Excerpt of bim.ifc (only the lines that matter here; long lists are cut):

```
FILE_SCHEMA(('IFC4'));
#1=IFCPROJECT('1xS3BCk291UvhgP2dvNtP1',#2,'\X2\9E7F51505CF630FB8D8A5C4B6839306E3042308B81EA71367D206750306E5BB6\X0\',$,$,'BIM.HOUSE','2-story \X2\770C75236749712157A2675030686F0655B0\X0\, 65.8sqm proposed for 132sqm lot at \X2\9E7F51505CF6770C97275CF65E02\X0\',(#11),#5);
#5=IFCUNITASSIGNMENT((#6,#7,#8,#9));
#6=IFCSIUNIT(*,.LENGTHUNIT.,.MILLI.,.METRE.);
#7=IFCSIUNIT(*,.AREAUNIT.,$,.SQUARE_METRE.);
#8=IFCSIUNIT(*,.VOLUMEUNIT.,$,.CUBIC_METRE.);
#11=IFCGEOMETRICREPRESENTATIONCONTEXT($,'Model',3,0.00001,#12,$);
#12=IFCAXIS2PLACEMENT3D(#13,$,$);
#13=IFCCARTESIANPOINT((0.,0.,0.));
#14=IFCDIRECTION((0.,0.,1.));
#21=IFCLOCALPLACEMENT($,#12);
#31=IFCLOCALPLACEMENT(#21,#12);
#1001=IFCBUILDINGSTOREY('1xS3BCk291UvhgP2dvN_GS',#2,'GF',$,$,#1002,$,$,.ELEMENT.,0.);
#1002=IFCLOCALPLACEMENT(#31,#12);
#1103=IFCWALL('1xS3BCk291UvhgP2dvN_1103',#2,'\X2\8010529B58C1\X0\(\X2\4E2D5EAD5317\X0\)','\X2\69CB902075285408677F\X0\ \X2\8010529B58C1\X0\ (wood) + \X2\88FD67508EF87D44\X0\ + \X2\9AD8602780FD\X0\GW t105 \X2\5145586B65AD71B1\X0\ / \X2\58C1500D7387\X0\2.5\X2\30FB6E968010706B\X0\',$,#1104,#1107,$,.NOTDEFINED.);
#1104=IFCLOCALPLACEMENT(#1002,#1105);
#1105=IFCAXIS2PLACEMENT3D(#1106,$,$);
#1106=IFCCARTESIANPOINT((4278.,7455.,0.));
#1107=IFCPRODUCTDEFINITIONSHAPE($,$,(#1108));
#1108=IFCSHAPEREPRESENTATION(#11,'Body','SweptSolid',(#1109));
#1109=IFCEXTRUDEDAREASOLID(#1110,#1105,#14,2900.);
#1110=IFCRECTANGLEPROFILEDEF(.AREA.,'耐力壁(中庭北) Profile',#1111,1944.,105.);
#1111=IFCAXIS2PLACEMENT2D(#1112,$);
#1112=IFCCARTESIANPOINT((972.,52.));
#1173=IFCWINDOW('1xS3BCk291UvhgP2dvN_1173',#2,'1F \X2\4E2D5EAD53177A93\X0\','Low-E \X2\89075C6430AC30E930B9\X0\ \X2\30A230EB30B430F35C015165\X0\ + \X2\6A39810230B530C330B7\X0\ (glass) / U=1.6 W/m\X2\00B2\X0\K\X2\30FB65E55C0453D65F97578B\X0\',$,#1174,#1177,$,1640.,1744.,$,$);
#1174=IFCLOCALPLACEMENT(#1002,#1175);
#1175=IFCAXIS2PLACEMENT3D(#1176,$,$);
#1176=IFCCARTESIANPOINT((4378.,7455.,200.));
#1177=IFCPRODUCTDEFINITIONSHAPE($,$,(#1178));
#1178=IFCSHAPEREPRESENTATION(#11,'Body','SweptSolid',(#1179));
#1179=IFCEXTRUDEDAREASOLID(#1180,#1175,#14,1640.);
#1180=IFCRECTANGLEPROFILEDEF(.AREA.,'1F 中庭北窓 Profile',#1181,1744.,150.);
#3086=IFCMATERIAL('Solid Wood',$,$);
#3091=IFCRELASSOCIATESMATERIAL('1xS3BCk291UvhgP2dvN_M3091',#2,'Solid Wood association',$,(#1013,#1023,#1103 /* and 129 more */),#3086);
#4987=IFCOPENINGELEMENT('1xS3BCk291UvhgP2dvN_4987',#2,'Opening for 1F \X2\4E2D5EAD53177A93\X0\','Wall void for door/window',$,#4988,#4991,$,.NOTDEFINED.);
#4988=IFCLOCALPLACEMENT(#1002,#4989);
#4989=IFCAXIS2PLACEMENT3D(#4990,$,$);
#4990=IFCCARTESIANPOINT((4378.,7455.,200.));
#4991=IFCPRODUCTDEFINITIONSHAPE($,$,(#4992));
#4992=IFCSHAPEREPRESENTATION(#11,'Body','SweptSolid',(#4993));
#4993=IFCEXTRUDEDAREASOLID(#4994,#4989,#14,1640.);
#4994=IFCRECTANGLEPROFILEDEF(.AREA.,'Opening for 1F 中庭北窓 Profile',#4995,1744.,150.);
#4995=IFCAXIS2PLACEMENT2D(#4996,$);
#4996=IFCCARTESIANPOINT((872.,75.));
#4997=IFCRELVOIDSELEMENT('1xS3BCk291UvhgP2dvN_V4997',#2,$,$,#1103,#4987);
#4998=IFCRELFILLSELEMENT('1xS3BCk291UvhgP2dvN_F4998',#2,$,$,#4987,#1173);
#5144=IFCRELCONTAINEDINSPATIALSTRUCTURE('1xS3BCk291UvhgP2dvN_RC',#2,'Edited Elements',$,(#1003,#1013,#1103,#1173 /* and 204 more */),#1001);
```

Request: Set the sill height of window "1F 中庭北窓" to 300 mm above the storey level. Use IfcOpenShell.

```python
import numpy as np
import ifcopenshell
import ifcopenshell.api.geometry
import ifcopenshell.geom
import ifcopenshell.util.element
import ifcopenshell.util.placement
import ifcopenshell.util.shape
import ifcopenshell.util.unit

model = ifcopenshell.open("bim.ifc")
unit_scale = ifcopenshell.util.unit.calculate_unit_scale(model)

window = model.by_guid("1xS3BCk291UvhgP2dvN_1173")
opening = window.FillsVoids[0].RelatingOpeningElement
storey = ifcopenshell.util.element.get_container(window, ifc_class="IfcBuildingStorey")
level = ifcopenshell.util.placement.get_local_placement(storey.ObjectPlacement)[2, 3]

# The opening's origin need not be at the sill, so measure its lowest point.
shape = ifcopenshell.geom.create_shape(ifcopenshell.geom.settings(), opening)
bottom = ifcopenshell.util.shape.get_shape_bottom_elevation(shape, shape.geometry) / unit_scale
dz = level + 0.3 / unit_scale - bottom

shift = np.array([0.0, 0.0, dz])
# The window is not placed relative to its opening, so move both.
for product in (opening, window):
    matrix = ifcopenshell.util.placement.get_local_placement(product.ObjectPlacement)
    matrix[:3, 3] += shift
    ifcopenshell.api.geometry.edit_object_placement(model, product=product, matrix=matrix, is_si=False)

print(f"moved by {dz * unit_scale:+.3f} m")

model.write("bim_updated.ifc")
```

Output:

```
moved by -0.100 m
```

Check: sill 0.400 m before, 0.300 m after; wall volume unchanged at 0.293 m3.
